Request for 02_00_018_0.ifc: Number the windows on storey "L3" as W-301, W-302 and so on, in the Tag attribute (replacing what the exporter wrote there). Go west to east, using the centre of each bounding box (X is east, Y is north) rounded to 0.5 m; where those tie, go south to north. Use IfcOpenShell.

First a look at what the model holds.

```python
import ifcopenshell
import ifcopenshell.util.element
import ifcopenshell.util.placement

model = ifcopenshell.open("02_00_018_0.ifc")
print(model.schema)
storey = next(s for s in model.by_type("IfcBuildingStorey") if s.Name == "L3")
windows = [e for e in ifcopenshell.util.element.get_decomposition(storey) if e.is_a("IfcWindow")]
for e in sorted(windows, key=lambda e: e.id()):
    origin = ifcopenshell.util.placement.get_local_placement(e.ObjectPlacement)[:3, 3]
    print(e.id(), e.Tag, e.Name, origin.round(2) + 0.0, sep=" | ")
```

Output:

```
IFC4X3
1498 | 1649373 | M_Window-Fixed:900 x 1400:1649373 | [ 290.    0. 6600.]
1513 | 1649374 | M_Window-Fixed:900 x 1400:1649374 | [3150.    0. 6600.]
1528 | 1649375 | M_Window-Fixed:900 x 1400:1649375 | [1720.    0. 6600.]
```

```python
import ifcopenshell
import ifcopenshell.geom
import ifcopenshell.util.element
import ifcopenshell.util.shape

model = ifcopenshell.open("02_00_018_0.ifc")
settings = ifcopenshell.geom.settings()
settings.set("use-world-coords", True)


def centre(element):
    shape = ifcopenshell.geom.create_shape(settings, element)
    return ifcopenshell.util.shape.get_bbox_centroid(shape.geometry)


storey = next(s for s in model.by_type("IfcBuildingStorey") if s.Name == "L3")
windows = [e for e in ifcopenshell.util.element.get_decomposition(storey) if e.is_a("IfcWindow")]

# Insertion points can sit at a corner or the storey origin, so sort by the geometry (in metres).
centres = {e: centre(e) for e in windows}
windows.sort(key=lambda e: (round(centres[e][0] / 0.5), centres[e][1]))

for i, e in enumerate(windows, start=1):
    number = f"W-3{i:02d}"
    e.Tag = number
    print(e.id(), number)

model.write("02_00_018_0_v2.ifc")
```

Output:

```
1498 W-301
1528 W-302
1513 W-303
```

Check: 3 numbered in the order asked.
